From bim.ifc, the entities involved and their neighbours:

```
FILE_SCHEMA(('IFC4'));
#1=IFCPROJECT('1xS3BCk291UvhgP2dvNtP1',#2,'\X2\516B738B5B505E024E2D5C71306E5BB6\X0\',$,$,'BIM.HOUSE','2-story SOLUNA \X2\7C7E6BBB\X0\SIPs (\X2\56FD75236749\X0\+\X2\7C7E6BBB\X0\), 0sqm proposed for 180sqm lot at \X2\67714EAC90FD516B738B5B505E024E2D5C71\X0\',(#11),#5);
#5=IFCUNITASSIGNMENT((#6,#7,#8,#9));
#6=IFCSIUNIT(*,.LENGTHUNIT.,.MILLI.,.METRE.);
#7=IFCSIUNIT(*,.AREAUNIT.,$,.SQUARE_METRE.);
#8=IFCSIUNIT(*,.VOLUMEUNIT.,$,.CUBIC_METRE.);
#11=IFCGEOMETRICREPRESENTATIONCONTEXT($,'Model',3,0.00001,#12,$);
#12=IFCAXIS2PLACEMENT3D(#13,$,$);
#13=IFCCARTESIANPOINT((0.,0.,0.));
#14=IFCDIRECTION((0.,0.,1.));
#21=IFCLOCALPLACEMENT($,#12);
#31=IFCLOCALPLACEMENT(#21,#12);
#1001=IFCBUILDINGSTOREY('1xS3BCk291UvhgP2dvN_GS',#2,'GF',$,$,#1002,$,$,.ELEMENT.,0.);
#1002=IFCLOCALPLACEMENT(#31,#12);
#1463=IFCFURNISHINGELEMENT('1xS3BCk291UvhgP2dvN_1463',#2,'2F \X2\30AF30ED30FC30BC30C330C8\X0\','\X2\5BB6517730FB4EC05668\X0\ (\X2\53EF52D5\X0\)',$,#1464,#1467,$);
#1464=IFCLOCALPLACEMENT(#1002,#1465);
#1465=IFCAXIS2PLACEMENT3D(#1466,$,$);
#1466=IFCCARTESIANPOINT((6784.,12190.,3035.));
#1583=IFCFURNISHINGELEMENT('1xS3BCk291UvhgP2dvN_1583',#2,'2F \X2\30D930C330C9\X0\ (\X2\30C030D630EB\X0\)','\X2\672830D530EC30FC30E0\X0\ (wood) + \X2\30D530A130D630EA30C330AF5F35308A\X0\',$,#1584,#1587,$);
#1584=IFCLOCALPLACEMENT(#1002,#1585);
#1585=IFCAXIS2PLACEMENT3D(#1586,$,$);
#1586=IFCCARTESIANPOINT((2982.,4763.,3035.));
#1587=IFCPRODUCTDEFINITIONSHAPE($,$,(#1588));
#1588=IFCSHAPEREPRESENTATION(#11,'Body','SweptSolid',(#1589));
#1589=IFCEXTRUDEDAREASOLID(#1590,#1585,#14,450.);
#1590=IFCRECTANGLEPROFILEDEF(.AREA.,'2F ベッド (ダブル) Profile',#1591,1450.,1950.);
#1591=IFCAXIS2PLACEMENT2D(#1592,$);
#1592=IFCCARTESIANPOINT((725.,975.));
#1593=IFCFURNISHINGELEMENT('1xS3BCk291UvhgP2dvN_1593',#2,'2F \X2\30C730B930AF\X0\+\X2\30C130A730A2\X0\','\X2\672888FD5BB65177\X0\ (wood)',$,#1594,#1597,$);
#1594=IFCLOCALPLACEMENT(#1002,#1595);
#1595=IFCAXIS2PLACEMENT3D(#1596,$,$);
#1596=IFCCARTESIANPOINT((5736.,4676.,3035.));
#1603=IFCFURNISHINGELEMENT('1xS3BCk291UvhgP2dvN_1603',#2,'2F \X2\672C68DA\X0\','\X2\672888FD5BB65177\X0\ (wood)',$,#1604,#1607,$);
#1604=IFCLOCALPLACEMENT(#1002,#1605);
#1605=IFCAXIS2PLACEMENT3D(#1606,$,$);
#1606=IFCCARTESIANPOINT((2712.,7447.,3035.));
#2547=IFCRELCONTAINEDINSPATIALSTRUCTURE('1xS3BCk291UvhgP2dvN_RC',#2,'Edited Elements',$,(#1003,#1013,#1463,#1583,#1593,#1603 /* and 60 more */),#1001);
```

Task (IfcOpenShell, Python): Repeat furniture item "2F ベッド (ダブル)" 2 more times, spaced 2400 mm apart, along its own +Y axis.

```python
import ifcopenshell
import ifcopenshell.api.geometry
import ifcopenshell.api.root
import ifcopenshell.util.element
import ifcopenshell.util.placement
import ifcopenshell.util.unit

model = ifcopenshell.open("bim.ifc")
unit_scale = ifcopenshell.util.unit.calculate_unit_scale(model)


def reuse_history(source, copy):
    """copy_class also copies each property set's owner history, people and application; keep the originals."""
    for rel in copy.IsDefinedBy:
        if rel.is_a("IfcRelDefinesByProperties") and (history := rel.RelatingPropertyDefinition.OwnerHistory):
            rel.RelatingPropertyDefinition.OwnerHistory = source.OwnerHistory
            ifcopenshell.util.element.remove_deep2(model, history)


source = model.by_id(1583)
base = ifcopenshell.util.placement.get_local_placement(source.ObjectPlacement)
step = base[:3, 1] * 2.4 / unit_scale

for i in range(1, 3):
    copy = ifcopenshell.api.root.copy_class(model, product=source)
    copy.Representation = ifcopenshell.util.element.copy_deep(
        model, source.Representation, exclude=["IfcGeometricRepresentationContext", "IfcRepresentationMap"]
    )
    reuse_history(source, copy)
    matrix = base.copy()
    matrix[:3, 3] += i * step
    print("added at", matrix[:3, 3].round(3) + 0.0)
    ifcopenshell.api.geometry.edit_object_placement(model, product=copy, matrix=matrix, is_si=False)

model.write("bim_rev.ifc")
```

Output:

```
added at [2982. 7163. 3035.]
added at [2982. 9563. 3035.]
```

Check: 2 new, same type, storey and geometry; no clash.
